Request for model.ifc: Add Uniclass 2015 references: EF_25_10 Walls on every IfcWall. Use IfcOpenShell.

First a look at what the model holds.

```python
import ifcopenshell

model = ifcopenshell.open("model.ifc")
print(model.schema)
print("classifications:", [c.Name for c in model.by_type("IfcClassification")])
for ifc_class in ("IfcDoor", "IfcRoof", "IfcStair", "IfcWall", "IfcWindow"):
    print(ifc_class, len(model.by_type(ifc_class)))
```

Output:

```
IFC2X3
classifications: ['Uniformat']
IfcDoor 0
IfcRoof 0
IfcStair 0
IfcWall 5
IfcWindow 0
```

```python
import ifcopenshell
import ifcopenshell.api.classification

model = ifcopenshell.open("model.ifc")

# IFC2X3 requires Source and Edition and has no link from the project to the system.
system = model.create_entity("IfcClassification", Source="NBS", Edition="2015", Name="Uniclass 2015")

codes = {
    "IfcWall": ("EF_25_10", "Walls"),
}
for ifc_class, (code, name) in codes.items():
    products = model.by_type(ifc_class)
    ifcopenshell.api.classification.add_reference(
        model, products=products, classification=system, identification=code, name=name
    )
    print(code, len(products))

model.write("model_v2.ifc")
```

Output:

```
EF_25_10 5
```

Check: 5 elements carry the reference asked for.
